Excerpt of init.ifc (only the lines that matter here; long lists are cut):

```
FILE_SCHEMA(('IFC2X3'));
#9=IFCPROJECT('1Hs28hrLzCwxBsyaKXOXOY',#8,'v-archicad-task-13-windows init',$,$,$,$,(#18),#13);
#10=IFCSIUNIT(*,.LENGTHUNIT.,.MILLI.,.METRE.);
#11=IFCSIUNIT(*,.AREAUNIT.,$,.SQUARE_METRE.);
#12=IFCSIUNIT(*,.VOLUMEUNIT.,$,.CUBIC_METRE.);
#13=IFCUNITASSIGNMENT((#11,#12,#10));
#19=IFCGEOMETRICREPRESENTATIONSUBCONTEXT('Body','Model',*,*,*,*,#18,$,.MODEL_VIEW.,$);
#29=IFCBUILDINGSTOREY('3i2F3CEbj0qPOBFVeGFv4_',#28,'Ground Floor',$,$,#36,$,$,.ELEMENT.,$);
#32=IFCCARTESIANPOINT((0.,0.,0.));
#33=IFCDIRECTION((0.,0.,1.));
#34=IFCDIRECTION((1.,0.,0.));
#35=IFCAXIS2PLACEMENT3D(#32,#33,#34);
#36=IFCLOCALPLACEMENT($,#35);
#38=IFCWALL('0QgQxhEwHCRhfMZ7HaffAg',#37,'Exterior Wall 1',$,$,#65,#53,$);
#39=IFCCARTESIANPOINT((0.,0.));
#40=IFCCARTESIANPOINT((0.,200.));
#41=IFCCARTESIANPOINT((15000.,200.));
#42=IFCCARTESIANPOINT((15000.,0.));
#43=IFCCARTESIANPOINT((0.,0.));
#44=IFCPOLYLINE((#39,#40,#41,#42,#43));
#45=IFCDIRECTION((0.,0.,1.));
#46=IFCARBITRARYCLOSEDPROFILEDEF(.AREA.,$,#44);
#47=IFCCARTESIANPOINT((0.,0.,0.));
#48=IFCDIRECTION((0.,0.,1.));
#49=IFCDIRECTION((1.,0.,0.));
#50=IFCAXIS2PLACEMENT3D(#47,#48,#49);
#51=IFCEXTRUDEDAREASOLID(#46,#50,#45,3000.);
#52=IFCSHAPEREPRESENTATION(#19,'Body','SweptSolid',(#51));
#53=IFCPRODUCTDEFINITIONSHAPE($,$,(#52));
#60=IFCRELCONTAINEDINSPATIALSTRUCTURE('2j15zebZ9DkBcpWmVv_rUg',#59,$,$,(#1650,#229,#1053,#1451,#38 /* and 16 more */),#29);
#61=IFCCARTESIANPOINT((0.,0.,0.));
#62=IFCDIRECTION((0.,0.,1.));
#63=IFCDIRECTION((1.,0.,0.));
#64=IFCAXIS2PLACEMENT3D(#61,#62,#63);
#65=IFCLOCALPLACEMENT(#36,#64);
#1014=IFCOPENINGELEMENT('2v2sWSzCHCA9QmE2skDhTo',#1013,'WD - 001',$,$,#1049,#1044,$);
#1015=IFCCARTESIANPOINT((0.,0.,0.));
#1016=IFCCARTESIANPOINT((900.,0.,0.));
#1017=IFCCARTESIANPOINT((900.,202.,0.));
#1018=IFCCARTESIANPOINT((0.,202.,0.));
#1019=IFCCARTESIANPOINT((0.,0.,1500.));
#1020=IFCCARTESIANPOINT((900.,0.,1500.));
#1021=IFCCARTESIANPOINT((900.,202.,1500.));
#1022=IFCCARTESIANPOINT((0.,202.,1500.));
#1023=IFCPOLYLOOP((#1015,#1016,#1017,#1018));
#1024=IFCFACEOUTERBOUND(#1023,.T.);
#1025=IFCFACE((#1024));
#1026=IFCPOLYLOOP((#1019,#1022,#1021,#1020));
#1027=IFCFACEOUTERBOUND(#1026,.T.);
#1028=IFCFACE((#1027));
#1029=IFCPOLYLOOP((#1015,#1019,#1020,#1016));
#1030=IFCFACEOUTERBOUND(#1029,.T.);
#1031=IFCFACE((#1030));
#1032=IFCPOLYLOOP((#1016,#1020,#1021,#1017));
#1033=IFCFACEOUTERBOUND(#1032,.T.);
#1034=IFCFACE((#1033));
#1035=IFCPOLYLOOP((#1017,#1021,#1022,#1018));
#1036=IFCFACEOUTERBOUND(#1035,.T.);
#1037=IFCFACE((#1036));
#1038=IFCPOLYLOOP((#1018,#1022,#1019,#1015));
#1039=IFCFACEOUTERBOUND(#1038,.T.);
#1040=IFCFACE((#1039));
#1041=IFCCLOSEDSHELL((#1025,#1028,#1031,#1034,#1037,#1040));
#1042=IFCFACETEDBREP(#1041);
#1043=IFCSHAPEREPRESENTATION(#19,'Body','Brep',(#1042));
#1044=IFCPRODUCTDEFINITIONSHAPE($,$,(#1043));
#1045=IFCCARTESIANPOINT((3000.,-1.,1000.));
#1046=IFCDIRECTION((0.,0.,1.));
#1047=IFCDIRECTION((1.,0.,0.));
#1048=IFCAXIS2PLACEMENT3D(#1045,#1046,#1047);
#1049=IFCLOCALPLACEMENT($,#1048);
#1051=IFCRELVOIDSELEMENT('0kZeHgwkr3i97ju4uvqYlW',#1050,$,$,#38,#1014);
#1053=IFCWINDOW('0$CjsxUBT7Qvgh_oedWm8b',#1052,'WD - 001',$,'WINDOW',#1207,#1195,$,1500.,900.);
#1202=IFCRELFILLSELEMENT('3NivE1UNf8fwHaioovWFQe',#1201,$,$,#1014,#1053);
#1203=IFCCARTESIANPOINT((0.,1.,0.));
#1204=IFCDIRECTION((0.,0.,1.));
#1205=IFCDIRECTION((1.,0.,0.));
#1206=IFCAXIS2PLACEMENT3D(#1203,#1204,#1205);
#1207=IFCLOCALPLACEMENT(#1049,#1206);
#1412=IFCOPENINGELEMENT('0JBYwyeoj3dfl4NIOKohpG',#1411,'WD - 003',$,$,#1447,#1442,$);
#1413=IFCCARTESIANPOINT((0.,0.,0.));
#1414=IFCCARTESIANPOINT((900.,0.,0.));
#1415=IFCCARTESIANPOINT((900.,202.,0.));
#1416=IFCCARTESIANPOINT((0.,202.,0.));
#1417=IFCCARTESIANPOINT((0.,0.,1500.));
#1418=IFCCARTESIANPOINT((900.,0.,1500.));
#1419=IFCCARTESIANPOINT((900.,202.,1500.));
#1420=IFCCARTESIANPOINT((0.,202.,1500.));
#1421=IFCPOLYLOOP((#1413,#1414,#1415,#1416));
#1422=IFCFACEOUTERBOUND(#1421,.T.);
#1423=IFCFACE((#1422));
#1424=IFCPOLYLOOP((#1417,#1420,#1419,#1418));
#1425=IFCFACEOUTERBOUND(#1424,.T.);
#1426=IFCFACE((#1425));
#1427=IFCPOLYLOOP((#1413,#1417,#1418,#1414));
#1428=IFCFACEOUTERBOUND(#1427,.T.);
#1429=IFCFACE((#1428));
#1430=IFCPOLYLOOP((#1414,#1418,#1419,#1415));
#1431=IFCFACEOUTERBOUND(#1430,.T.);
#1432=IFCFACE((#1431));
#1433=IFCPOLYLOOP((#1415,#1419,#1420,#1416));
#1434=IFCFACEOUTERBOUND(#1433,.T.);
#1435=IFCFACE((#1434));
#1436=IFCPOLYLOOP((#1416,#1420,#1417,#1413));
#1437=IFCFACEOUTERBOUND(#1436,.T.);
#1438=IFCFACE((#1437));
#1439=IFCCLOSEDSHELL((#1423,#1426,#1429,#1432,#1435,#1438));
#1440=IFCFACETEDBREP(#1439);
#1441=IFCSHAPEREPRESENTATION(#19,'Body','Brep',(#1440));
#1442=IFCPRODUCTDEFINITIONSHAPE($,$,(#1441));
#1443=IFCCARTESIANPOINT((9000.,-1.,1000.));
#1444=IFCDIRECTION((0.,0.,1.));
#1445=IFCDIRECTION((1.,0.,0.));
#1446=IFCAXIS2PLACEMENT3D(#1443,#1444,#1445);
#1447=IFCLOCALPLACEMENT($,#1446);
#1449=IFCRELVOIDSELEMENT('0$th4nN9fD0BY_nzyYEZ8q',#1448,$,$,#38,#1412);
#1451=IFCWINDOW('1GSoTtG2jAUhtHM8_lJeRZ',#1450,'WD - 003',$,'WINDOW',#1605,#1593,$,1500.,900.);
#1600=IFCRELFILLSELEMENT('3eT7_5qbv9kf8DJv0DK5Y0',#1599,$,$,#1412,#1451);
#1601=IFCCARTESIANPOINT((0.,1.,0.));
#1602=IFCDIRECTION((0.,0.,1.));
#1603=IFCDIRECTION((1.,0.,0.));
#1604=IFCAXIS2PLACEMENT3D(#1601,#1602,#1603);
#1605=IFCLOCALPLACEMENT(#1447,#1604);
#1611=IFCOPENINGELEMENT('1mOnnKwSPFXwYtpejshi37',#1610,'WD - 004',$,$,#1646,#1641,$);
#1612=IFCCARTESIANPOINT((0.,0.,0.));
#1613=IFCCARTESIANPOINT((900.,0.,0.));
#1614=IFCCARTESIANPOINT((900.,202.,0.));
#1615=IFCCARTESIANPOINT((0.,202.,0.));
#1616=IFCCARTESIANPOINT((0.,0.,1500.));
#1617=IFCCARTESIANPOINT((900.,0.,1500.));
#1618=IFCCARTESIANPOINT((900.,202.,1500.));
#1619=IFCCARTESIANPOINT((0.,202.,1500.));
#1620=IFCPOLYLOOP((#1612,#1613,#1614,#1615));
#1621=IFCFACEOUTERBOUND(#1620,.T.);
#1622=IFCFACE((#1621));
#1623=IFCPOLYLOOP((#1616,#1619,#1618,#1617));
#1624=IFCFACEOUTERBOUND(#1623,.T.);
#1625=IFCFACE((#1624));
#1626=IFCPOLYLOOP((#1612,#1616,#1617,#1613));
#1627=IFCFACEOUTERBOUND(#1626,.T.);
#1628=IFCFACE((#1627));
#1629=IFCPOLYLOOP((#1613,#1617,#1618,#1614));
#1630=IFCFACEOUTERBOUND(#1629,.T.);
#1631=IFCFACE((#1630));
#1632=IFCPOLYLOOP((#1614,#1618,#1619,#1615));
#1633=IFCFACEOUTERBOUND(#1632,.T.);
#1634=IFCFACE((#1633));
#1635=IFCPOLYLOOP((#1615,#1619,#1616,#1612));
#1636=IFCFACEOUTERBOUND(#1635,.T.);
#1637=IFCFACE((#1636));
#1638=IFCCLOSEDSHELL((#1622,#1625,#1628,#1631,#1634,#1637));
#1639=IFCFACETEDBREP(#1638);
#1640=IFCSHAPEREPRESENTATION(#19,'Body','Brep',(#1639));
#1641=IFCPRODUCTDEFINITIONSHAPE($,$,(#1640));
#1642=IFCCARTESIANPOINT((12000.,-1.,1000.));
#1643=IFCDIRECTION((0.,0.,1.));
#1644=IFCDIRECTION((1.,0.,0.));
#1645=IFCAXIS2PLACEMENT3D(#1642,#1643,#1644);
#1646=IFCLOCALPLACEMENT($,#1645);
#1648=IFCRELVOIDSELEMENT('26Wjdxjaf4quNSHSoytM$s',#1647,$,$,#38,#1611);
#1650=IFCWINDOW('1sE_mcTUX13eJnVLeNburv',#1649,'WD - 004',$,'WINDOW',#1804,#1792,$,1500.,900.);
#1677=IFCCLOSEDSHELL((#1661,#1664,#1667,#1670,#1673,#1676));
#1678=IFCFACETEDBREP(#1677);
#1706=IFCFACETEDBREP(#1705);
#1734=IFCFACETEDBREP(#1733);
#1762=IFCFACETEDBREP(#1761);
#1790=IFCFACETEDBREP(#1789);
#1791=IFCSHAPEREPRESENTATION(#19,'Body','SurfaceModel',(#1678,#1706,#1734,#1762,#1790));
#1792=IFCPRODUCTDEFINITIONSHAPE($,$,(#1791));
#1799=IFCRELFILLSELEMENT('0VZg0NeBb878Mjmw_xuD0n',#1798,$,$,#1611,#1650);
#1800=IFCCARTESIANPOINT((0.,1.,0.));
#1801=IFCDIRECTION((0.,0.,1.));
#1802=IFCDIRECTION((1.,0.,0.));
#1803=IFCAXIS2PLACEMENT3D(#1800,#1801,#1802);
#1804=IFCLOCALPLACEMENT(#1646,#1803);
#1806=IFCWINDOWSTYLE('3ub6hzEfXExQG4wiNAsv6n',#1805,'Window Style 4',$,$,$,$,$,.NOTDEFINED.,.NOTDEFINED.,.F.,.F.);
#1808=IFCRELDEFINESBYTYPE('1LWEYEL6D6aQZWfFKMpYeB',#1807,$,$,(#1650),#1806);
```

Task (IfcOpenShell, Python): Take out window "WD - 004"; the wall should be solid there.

```python
import ifcopenshell
import ifcopenshell.api.feature
import ifcopenshell.api.root
import ifcopenshell.geom
import ifcopenshell.util.shape

model = ifcopenshell.open("init.ifc")
settings = ifcopenshell.geom.settings()


def volume(element):
    """Net volume in cubic metres, openings subtracted."""
    shape = ifcopenshell.geom.create_shape(settings, element)
    return ifcopenshell.util.shape.get_volume(shape.geometry)


window = model.by_guid("1sE_mcTUX13eJnVLeNburv")
opening = window.FillsVoids[0].RelatingOpeningElement
wall = opening.VoidsElements[0].RelatingBuildingElement
before = volume(wall)

ifcopenshell.api.root.remove_product(model, product=window)
ifcopenshell.api.feature.remove_feature(model, feature=opening)

after = volume(wall)

print(f"wall volume {before:.3f} -> {after:.3f} m3")

model.write("init_v2.ifc")
```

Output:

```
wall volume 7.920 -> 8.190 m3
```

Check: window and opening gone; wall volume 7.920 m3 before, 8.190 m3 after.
